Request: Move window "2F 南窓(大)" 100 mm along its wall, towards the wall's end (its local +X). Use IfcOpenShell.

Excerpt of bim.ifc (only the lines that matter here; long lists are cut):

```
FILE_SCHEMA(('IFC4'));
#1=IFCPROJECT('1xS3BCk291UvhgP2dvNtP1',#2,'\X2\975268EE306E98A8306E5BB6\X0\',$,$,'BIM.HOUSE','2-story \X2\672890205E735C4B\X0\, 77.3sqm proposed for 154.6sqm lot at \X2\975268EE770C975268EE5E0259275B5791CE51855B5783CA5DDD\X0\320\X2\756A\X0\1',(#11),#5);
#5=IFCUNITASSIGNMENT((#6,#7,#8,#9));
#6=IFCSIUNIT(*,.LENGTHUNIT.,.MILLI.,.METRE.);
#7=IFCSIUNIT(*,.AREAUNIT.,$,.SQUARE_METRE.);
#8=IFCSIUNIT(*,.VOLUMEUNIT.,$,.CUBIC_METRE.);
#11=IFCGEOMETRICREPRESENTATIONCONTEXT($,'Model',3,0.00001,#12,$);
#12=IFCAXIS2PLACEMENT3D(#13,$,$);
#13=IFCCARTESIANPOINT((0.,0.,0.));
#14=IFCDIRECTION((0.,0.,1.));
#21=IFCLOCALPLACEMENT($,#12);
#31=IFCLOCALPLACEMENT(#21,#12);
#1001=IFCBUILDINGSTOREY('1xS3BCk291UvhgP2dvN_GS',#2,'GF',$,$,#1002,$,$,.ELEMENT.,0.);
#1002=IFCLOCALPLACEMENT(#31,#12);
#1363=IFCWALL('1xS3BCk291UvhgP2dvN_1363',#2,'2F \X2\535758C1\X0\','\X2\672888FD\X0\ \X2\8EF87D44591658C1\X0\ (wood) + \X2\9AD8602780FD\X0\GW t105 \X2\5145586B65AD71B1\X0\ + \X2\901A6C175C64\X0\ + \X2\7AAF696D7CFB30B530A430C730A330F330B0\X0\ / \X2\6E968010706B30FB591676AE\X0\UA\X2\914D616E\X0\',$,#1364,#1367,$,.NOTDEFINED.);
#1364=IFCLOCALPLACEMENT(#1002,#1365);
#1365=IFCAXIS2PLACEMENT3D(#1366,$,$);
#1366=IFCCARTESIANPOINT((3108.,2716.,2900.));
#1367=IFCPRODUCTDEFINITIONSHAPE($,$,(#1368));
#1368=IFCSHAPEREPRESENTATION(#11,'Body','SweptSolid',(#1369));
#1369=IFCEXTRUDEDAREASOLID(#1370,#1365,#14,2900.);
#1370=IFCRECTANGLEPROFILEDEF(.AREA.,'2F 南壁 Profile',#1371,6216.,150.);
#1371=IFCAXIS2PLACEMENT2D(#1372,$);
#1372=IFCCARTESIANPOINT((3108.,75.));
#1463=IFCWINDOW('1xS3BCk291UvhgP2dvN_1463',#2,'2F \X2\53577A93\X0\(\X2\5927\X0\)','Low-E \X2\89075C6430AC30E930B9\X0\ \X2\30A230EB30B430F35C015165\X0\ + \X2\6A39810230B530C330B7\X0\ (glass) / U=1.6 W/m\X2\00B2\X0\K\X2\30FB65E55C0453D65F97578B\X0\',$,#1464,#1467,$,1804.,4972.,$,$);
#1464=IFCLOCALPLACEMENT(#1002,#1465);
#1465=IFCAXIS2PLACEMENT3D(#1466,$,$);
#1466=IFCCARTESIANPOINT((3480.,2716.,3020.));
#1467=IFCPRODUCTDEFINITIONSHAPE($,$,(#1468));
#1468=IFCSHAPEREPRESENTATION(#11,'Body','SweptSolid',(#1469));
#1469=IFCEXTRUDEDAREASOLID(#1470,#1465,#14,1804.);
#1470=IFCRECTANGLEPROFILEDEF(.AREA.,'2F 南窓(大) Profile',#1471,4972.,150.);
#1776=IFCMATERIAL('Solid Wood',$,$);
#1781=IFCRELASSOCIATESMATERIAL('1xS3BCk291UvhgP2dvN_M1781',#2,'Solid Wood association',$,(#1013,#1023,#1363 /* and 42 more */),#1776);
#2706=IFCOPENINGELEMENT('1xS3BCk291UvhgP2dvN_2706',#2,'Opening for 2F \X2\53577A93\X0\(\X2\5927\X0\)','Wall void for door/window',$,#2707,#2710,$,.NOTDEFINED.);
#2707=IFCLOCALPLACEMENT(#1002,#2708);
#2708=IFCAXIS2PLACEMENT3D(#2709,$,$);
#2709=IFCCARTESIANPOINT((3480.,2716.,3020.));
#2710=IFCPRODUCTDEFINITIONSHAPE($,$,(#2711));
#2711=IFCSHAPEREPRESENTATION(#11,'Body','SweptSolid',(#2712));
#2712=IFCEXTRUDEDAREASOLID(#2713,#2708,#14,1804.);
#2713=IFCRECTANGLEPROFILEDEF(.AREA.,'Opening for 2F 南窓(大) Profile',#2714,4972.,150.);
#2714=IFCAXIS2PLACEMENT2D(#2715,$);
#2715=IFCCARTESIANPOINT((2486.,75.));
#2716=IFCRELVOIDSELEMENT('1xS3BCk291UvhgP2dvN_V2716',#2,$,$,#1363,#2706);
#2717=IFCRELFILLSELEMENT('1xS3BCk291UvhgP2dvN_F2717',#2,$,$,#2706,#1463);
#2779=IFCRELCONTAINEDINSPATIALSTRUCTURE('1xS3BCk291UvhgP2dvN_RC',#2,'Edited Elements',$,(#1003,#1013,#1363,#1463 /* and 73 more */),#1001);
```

```python
import ifcopenshell
import ifcopenshell.api.geometry
import ifcopenshell.util.placement
import ifcopenshell.util.unit

model = ifcopenshell.open("bim.ifc")
unit_scale = ifcopenshell.util.unit.calculate_unit_scale(model)

window = model.by_guid("1xS3BCk291UvhgP2dvN_1463")
opening = window.FillsVoids[0].RelatingOpeningElement
wall = opening.VoidsElements[0].RelatingBuildingElement

wall_matrix = ifcopenshell.util.placement.get_local_placement(wall.ObjectPlacement)
shift = wall_matrix[:3, 0] * 0.1 / unit_scale
before = ifcopenshell.util.placement.get_local_placement(window.ObjectPlacement)[:3, 3].copy()

# The window is not placed relative to its opening, so move both.
for product in (opening, window):
    matrix = ifcopenshell.util.placement.get_local_placement(product.ObjectPlacement)
    matrix[:3, 3] += shift
    ifcopenshell.api.geometry.edit_object_placement(model, product=product, matrix=matrix, is_si=False)

after = ifcopenshell.util.placement.get_local_placement(window.ObjectPlacement)[:3, 3]
print("window moved by", (after - before).round(3) + 0.0)

model.write("bim-out.ifc")
```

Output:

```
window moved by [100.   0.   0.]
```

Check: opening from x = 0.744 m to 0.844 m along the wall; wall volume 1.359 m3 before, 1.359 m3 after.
